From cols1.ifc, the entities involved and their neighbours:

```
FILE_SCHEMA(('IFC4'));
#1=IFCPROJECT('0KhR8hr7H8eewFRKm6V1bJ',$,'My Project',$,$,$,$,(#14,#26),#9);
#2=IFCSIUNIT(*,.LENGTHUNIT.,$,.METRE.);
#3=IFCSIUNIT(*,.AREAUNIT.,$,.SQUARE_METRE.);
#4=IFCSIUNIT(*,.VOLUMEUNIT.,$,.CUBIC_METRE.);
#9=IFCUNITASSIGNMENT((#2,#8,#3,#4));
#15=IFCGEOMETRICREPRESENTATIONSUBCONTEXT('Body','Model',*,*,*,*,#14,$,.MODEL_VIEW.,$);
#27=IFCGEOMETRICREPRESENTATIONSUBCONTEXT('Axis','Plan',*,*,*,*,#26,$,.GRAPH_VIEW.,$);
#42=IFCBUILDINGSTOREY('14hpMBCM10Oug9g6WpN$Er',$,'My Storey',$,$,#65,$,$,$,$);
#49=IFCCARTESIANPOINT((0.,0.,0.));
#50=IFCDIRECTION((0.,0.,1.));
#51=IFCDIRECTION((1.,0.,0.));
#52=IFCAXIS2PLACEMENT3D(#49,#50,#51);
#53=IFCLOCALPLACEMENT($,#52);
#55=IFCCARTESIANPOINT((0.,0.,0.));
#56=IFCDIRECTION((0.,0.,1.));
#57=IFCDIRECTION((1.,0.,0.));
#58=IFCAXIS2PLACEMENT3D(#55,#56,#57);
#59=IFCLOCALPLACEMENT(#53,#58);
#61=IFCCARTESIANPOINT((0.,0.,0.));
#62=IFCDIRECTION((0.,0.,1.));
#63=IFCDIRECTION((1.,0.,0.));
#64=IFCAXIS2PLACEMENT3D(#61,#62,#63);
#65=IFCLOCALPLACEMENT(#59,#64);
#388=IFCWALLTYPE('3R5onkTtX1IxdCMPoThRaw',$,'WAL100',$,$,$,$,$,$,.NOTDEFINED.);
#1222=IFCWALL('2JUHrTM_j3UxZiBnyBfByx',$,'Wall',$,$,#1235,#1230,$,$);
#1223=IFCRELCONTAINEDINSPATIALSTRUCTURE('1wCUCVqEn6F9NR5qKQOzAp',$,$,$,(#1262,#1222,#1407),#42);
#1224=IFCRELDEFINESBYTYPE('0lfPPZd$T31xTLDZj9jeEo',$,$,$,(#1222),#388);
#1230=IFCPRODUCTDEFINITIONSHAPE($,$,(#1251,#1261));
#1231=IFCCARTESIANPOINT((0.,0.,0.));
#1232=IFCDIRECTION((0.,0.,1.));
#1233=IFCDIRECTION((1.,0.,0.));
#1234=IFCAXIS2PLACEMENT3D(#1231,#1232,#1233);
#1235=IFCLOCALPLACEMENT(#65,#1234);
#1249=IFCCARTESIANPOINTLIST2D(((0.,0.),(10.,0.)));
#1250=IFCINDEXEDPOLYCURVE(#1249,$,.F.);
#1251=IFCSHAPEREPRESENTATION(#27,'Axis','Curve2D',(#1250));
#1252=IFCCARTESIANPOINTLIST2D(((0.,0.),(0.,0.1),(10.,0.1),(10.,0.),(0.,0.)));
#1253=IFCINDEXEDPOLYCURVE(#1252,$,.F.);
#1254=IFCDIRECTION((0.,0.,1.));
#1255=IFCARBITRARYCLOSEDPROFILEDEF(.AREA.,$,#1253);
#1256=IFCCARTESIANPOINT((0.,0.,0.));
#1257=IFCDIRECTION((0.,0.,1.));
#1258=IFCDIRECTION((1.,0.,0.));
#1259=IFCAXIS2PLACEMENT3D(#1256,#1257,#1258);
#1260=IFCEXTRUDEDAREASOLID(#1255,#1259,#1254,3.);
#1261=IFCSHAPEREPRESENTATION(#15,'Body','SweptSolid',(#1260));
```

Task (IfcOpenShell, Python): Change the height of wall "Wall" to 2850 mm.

```python
import ifcopenshell
import ifcopenshell.geom
import ifcopenshell.util.representation
import ifcopenshell.util.shape
import ifcopenshell.util.unit

model = ifcopenshell.open("cols1.ifc")
unit_scale = ifcopenshell.util.unit.calculate_unit_scale(model)
settings = ifcopenshell.geom.settings()


def volume(element):
    """Net volume in cubic metres, openings subtracted."""
    shape = ifcopenshell.geom.create_shape(settings, element)
    return ifcopenshell.util.shape.get_volume(shape.geometry)


wall = model.by_guid("2JUHrTM_j3UxZiBnyBfByx")
before = volume(wall)

body = ifcopenshell.util.representation.get_representation(wall, "Model", "Body")
solid = body.Items[0]
old_height = solid.Depth
solid.Depth = 2.85 / unit_scale
after = volume(wall)

print(f"height {old_height:g} -> {solid.Depth:g}, volume {before:.3f} -> {after:.3f} m3")

model.write("cols1_v2.ifc")
```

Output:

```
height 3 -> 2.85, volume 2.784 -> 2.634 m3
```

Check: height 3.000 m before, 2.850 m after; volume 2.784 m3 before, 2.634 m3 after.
